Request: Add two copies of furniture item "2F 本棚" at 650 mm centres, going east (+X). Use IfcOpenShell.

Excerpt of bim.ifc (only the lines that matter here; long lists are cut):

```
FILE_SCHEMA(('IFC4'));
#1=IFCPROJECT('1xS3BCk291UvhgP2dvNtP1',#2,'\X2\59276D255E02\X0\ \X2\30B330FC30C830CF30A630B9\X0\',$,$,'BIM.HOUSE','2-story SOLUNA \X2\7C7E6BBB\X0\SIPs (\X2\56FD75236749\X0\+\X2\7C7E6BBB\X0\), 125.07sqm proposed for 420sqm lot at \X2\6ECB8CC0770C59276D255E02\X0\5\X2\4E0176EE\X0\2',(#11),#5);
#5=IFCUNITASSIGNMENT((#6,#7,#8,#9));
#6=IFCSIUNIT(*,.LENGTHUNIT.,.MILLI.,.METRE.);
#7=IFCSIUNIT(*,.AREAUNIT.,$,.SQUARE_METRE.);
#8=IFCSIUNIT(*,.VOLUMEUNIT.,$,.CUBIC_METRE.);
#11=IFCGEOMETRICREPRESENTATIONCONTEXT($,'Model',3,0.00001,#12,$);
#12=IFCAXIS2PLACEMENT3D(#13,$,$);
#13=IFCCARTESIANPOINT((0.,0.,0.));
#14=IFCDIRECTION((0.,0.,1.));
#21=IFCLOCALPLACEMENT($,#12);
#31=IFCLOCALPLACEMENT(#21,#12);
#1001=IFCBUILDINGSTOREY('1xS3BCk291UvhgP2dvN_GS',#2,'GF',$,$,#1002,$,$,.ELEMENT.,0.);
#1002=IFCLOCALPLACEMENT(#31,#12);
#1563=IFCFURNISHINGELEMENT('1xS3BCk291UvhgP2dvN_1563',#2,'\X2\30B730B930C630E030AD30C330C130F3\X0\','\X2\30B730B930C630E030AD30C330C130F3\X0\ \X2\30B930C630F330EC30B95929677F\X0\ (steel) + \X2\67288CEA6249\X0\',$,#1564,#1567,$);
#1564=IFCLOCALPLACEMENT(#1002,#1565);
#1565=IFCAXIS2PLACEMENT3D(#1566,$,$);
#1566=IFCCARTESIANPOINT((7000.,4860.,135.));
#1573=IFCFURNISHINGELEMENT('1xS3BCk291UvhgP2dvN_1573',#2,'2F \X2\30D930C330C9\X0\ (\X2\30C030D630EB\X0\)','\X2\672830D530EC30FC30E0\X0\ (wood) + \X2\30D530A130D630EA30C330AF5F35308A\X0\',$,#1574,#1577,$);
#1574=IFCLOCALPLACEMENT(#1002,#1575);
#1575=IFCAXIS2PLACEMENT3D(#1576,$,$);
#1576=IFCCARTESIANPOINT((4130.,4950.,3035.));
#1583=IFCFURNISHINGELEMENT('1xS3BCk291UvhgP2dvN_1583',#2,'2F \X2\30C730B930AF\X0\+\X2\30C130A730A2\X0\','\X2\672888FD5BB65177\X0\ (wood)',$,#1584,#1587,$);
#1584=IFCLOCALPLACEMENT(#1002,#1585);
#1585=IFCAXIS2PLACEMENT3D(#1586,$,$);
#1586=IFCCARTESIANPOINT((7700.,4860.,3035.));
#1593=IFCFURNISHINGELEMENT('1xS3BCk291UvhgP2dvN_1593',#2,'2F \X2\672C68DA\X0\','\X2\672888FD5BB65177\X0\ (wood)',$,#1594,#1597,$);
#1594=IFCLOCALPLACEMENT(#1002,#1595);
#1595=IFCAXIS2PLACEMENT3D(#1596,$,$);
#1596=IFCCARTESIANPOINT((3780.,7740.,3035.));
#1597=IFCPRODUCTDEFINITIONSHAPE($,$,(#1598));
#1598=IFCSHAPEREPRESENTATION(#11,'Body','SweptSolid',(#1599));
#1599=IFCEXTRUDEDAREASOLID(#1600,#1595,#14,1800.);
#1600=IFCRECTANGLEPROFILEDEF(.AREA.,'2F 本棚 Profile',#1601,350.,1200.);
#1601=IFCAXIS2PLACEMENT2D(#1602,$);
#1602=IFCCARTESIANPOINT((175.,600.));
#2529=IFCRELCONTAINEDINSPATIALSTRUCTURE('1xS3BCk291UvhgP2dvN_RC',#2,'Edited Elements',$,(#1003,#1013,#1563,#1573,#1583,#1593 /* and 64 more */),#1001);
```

```python
import numpy as np
import ifcopenshell
import ifcopenshell.api.geometry
import ifcopenshell.api.root
import ifcopenshell.util.element
import ifcopenshell.util.placement

model = ifcopenshell.open("bim.ifc")


def reuse_history(source, copy):
    """copy_class also copies each property set's owner history, people and application; keep the originals."""
    for rel in copy.IsDefinedBy:
        if rel.is_a("IfcRelDefinesByProperties") and (history := rel.RelatingPropertyDefinition.OwnerHistory):
            rel.RelatingPropertyDefinition.OwnerHistory = source.OwnerHistory
            ifcopenshell.util.element.remove_deep2(model, history)


source = model.by_id(1593)
base = ifcopenshell.util.placement.get_local_placement(source.ObjectPlacement)
step = np.array([1.0, 0.0, 0.0]) * 650.0

for i in range(1, 3):
    copy = ifcopenshell.api.root.copy_class(model, product=source)
    copy.Representation = ifcopenshell.util.element.copy_deep(
        model, source.Representation, exclude=["IfcGeometricRepresentationContext", "IfcRepresentationMap"]
    )
    reuse_history(source, copy)
    matrix = base.copy()
    matrix[:3, 3] += i * step
    print("added at", matrix[:3, 3].round(3) + 0.0)
    ifcopenshell.api.geometry.edit_object_placement(model, product=copy, matrix=matrix, is_si=False)

model.write("bim_edited.ifc")
```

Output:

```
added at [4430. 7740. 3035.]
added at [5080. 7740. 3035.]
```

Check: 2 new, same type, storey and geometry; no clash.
